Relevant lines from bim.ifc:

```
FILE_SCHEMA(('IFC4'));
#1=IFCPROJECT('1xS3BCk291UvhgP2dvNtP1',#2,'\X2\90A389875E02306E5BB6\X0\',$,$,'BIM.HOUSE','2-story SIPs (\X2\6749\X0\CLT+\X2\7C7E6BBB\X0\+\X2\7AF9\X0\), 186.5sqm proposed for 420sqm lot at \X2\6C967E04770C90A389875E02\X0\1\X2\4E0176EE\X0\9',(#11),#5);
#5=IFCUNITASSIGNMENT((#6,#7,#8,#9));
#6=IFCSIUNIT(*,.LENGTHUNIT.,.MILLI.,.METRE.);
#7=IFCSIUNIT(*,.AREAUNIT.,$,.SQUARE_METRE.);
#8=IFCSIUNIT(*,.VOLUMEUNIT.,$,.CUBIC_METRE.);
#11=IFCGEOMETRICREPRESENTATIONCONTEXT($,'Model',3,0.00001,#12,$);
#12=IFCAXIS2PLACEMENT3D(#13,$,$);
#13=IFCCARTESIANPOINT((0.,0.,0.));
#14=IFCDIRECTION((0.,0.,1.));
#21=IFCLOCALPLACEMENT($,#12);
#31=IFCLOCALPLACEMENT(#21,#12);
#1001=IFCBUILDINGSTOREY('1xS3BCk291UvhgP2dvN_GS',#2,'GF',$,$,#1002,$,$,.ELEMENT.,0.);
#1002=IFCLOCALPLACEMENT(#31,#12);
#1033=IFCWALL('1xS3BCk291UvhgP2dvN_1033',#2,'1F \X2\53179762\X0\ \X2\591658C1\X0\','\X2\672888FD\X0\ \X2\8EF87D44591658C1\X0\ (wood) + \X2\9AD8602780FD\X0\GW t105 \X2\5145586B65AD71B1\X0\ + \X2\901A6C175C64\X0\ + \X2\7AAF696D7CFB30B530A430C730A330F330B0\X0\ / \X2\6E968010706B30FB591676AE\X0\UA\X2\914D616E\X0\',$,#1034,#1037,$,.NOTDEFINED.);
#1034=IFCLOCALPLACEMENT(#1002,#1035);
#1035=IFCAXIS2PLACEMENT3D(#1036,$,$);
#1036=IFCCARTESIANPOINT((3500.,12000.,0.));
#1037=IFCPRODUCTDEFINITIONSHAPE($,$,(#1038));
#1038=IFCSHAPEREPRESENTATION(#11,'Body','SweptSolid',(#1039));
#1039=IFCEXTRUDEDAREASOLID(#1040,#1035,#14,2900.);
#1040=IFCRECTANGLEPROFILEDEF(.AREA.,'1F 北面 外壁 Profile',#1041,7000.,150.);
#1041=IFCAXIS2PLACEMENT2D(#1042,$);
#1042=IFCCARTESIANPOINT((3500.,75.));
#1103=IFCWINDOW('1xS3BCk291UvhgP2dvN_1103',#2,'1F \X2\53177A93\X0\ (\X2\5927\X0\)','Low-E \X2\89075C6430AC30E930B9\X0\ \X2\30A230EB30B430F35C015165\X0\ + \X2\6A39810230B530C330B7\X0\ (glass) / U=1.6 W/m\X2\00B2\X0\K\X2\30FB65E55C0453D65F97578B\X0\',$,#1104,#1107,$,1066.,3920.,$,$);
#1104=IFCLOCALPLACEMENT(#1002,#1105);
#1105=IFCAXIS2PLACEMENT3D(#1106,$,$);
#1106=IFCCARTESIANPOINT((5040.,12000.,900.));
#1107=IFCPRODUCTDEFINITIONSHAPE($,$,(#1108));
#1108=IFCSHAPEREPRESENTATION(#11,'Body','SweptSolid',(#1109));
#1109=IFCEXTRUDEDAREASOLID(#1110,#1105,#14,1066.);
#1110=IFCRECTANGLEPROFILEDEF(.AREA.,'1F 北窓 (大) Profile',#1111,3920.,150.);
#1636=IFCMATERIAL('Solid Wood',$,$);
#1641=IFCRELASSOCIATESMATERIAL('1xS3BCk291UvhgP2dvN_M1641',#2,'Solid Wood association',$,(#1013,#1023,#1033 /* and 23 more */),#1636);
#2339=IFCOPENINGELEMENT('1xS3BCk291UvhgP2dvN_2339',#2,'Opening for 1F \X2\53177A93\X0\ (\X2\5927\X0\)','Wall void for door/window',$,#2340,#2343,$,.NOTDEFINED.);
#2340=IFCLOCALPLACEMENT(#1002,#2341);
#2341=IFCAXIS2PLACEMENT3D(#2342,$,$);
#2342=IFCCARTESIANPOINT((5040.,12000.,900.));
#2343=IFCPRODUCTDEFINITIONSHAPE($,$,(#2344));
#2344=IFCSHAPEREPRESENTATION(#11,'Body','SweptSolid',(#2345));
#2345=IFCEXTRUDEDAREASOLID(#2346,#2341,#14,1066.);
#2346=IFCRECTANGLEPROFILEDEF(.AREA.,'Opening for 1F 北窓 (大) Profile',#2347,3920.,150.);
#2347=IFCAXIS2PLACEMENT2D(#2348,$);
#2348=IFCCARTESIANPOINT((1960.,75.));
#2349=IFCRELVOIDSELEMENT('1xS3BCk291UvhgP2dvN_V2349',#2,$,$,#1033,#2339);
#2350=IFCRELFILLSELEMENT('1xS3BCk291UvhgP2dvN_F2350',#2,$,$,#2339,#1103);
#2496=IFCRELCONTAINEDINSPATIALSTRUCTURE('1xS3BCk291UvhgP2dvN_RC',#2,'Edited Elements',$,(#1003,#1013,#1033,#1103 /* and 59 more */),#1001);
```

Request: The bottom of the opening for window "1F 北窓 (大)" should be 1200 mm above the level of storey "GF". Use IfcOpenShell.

```python
import numpy as np
import ifcopenshell
import ifcopenshell.api.geometry
import ifcopenshell.geom
import ifcopenshell.util.element
import ifcopenshell.util.placement
import ifcopenshell.util.shape
import ifcopenshell.util.unit

model = ifcopenshell.open("bim.ifc")
unit_scale = ifcopenshell.util.unit.calculate_unit_scale(model)

window = model.by_id(1103)
opening = window.FillsVoids[0].RelatingOpeningElement
storey = ifcopenshell.util.element.get_container(window, ifc_class="IfcBuildingStorey")
level = ifcopenshell.util.placement.get_local_placement(storey.ObjectPlacement)[2, 3]

# The opening's origin need not be at the sill, so measure its lowest point.
shape = ifcopenshell.geom.create_shape(ifcopenshell.geom.settings(), opening)
bottom = ifcopenshell.util.shape.get_shape_bottom_elevation(shape, shape.geometry) / unit_scale
dz = level + 1200.0 - bottom

shift = np.array([0.0, 0.0, dz])
# The window is not placed relative to its opening, so move both.
for product in (opening, window):
    matrix = ifcopenshell.util.placement.get_local_placement(product.ObjectPlacement)
    matrix[:3, 3] += shift
    ifcopenshell.api.geometry.edit_object_placement(model, product=product, matrix=matrix, is_si=False)

print(f"moved by {dz * unit_scale:+.3f} m")

model.write("bim_v2.ifc")
```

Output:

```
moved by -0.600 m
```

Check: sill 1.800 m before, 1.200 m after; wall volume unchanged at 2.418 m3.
